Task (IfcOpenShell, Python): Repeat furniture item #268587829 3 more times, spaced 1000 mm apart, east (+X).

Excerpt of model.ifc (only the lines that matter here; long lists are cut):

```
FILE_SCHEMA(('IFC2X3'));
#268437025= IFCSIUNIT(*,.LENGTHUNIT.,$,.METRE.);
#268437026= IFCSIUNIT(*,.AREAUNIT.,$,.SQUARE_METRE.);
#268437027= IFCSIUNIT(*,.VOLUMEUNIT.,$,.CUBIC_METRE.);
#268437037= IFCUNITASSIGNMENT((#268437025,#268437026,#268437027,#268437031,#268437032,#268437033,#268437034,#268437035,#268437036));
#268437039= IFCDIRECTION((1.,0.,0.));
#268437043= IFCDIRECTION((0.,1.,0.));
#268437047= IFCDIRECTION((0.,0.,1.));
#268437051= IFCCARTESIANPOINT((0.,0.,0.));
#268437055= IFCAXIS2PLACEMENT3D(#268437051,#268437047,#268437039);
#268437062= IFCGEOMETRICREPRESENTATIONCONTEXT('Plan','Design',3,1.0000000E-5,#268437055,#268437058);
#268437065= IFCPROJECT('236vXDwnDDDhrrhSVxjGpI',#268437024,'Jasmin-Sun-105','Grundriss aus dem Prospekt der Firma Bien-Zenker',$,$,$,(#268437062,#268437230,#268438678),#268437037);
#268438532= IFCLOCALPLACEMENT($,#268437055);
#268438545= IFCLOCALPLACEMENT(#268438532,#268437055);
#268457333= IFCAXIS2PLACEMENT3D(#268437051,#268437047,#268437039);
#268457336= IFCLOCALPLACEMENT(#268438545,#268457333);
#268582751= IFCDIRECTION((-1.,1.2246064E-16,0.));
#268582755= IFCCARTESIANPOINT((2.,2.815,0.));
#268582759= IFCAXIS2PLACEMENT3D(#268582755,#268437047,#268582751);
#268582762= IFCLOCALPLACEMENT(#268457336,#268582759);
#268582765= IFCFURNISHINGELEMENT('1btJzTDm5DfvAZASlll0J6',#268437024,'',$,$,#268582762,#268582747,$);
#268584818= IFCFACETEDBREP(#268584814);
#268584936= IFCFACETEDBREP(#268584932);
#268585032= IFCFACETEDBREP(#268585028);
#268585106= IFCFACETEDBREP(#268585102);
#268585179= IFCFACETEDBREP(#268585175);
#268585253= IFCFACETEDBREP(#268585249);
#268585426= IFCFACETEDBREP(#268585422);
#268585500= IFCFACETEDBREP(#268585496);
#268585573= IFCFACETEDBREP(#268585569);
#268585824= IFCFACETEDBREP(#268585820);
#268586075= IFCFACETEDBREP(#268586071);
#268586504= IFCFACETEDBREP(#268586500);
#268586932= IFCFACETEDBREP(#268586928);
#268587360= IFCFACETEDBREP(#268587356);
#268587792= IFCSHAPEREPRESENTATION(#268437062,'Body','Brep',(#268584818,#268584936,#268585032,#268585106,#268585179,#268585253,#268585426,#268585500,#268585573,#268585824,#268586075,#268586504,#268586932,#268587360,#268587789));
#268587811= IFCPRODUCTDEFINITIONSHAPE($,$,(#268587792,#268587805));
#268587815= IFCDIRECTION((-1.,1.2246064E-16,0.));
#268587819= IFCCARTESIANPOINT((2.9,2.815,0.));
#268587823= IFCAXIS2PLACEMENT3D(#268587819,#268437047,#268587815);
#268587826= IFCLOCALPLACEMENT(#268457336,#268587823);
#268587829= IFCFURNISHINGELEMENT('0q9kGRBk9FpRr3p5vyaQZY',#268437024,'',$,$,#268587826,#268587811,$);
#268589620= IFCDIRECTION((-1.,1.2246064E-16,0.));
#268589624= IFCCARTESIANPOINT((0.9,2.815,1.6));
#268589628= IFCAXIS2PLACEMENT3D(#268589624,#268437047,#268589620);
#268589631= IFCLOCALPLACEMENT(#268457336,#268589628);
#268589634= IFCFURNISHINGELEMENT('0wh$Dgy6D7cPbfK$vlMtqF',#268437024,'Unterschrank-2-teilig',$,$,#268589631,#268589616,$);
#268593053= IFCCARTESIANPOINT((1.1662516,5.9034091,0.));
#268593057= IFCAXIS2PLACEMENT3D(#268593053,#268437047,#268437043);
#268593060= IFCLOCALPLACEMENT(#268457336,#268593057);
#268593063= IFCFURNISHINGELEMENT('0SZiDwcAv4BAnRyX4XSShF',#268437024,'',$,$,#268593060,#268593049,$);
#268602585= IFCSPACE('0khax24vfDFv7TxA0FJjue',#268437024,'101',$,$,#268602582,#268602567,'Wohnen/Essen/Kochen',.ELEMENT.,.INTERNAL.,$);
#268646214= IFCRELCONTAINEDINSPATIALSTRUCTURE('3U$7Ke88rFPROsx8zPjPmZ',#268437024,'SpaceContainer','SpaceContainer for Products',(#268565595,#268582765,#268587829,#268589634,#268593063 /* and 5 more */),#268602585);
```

```python
import numpy as np
import ifcopenshell
import ifcopenshell.api.geometry
import ifcopenshell.api.root
import ifcopenshell.util.element
import ifcopenshell.util.placement
import ifcopenshell.util.unit

model = ifcopenshell.open("model.ifc")
unit_scale = ifcopenshell.util.unit.calculate_unit_scale(model)


def reuse_history(source, copy):
    """copy_class also copies each property set's owner history, people and application; keep the originals."""
    for rel in copy.IsDefinedBy:
        if rel.is_a("IfcRelDefinesByProperties") and (history := rel.RelatingPropertyDefinition.OwnerHistory):
            rel.RelatingPropertyDefinition.OwnerHistory = source.OwnerHistory
            ifcopenshell.util.element.remove_deep2(model, history)


source = model.by_guid("0q9kGRBk9FpRr3p5vyaQZY")
base = ifcopenshell.util.placement.get_local_placement(source.ObjectPlacement)
step = np.array([1.0, 0.0, 0.0]) * 1 / unit_scale

for i in range(1, 4):
    copy = ifcopenshell.api.root.copy_class(model, product=source)
    copy.Representation = ifcopenshell.util.element.copy_deep(
        model, source.Representation, exclude=["IfcGeometricRepresentationContext", "IfcRepresentationMap"]
    )
    reuse_history(source, copy)
    matrix = base.copy()
    matrix[:3, 3] += i * step
    print("added at", matrix[:3, 3].round(3) + 0.0)
    ifcopenshell.api.geometry.edit_object_placement(model, product=copy, matrix=matrix, is_si=False)

model.write("model_rev.ifc")
```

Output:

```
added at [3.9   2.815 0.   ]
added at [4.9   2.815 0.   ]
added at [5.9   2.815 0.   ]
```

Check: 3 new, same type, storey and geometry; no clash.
